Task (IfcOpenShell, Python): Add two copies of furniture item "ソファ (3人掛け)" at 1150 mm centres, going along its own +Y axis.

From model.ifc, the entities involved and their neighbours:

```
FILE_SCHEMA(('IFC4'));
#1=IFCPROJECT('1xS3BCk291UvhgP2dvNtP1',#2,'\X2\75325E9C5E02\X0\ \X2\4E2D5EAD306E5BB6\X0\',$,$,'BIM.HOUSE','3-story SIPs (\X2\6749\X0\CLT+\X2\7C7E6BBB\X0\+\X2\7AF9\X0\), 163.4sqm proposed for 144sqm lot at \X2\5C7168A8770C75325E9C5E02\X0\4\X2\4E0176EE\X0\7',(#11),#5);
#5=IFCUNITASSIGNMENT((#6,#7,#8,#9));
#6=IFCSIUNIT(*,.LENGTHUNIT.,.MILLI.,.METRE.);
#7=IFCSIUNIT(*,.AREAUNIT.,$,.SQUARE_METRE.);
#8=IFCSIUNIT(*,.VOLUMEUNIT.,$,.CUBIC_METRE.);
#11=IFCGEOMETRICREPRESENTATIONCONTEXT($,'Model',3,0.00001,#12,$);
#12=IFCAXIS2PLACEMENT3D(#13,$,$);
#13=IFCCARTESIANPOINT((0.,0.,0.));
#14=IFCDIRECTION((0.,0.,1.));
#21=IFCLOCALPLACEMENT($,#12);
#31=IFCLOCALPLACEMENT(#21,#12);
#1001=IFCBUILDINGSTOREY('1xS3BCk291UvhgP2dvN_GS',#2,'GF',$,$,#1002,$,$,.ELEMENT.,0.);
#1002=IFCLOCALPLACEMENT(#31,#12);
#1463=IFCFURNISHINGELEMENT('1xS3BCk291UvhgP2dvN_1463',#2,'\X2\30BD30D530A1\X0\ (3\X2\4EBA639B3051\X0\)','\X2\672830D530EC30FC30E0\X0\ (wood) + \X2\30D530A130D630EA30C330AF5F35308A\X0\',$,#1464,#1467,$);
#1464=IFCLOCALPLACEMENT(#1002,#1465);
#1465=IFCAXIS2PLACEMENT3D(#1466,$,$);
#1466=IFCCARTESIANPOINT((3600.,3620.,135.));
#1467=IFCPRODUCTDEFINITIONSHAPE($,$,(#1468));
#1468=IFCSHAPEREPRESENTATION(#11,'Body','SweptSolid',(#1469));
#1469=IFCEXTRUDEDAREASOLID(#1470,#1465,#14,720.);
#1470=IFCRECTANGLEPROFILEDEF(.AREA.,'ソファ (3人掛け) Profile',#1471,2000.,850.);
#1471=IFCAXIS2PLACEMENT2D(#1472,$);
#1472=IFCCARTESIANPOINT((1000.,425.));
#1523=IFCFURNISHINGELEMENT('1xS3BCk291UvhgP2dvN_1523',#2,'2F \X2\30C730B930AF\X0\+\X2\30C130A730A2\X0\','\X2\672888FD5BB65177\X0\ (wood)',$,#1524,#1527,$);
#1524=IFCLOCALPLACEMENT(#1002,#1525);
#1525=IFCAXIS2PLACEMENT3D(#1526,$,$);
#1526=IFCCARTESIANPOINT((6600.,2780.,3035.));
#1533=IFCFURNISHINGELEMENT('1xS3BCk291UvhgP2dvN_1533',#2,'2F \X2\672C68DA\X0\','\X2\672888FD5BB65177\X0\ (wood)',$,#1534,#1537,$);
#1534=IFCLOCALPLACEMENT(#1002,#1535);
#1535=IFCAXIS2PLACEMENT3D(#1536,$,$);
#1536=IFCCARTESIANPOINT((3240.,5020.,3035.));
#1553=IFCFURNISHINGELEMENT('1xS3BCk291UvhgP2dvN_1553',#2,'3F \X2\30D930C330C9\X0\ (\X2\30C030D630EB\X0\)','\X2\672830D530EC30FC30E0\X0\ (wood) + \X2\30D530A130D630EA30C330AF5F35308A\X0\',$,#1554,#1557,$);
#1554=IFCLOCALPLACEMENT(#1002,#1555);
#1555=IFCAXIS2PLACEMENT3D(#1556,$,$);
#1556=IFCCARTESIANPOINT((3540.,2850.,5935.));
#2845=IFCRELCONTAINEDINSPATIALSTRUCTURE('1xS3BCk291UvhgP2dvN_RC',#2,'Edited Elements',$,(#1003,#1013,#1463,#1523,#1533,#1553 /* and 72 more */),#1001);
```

```python
import ifcopenshell
import ifcopenshell.api.geometry
import ifcopenshell.api.root
import ifcopenshell.util.element
import ifcopenshell.util.placement

model = ifcopenshell.open("model.ifc")


def reuse_history(source, copy):
    """copy_class also copies each property set's owner history, people and application; keep the originals."""
    for rel in copy.IsDefinedBy:
        if rel.is_a("IfcRelDefinesByProperties") and (history := rel.RelatingPropertyDefinition.OwnerHistory):
            rel.RelatingPropertyDefinition.OwnerHistory = source.OwnerHistory
            ifcopenshell.util.element.remove_deep2(model, history)


source = model.by_id(1463)
base = ifcopenshell.util.placement.get_local_placement(source.ObjectPlacement)
step = base[:3, 1] * 1150.0

for i in range(1, 3):
    copy = ifcopenshell.api.root.copy_class(model, product=source)
    copy.Representation = ifcopenshell.util.element.copy_deep(
        model, source.Representation, exclude=["IfcGeometricRepresentationContext", "IfcRepresentationMap"]
    )
    reuse_history(source, copy)
    matrix = base.copy()
    matrix[:3, 3] += i * step
    print("added at", matrix[:3, 3].round(3) + 0.0)
    ifcopenshell.api.geometry.edit_object_placement(model, product=copy, matrix=matrix, is_si=False)

model.write("model_v2.ifc")
```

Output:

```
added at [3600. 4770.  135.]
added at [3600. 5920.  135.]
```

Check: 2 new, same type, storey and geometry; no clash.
